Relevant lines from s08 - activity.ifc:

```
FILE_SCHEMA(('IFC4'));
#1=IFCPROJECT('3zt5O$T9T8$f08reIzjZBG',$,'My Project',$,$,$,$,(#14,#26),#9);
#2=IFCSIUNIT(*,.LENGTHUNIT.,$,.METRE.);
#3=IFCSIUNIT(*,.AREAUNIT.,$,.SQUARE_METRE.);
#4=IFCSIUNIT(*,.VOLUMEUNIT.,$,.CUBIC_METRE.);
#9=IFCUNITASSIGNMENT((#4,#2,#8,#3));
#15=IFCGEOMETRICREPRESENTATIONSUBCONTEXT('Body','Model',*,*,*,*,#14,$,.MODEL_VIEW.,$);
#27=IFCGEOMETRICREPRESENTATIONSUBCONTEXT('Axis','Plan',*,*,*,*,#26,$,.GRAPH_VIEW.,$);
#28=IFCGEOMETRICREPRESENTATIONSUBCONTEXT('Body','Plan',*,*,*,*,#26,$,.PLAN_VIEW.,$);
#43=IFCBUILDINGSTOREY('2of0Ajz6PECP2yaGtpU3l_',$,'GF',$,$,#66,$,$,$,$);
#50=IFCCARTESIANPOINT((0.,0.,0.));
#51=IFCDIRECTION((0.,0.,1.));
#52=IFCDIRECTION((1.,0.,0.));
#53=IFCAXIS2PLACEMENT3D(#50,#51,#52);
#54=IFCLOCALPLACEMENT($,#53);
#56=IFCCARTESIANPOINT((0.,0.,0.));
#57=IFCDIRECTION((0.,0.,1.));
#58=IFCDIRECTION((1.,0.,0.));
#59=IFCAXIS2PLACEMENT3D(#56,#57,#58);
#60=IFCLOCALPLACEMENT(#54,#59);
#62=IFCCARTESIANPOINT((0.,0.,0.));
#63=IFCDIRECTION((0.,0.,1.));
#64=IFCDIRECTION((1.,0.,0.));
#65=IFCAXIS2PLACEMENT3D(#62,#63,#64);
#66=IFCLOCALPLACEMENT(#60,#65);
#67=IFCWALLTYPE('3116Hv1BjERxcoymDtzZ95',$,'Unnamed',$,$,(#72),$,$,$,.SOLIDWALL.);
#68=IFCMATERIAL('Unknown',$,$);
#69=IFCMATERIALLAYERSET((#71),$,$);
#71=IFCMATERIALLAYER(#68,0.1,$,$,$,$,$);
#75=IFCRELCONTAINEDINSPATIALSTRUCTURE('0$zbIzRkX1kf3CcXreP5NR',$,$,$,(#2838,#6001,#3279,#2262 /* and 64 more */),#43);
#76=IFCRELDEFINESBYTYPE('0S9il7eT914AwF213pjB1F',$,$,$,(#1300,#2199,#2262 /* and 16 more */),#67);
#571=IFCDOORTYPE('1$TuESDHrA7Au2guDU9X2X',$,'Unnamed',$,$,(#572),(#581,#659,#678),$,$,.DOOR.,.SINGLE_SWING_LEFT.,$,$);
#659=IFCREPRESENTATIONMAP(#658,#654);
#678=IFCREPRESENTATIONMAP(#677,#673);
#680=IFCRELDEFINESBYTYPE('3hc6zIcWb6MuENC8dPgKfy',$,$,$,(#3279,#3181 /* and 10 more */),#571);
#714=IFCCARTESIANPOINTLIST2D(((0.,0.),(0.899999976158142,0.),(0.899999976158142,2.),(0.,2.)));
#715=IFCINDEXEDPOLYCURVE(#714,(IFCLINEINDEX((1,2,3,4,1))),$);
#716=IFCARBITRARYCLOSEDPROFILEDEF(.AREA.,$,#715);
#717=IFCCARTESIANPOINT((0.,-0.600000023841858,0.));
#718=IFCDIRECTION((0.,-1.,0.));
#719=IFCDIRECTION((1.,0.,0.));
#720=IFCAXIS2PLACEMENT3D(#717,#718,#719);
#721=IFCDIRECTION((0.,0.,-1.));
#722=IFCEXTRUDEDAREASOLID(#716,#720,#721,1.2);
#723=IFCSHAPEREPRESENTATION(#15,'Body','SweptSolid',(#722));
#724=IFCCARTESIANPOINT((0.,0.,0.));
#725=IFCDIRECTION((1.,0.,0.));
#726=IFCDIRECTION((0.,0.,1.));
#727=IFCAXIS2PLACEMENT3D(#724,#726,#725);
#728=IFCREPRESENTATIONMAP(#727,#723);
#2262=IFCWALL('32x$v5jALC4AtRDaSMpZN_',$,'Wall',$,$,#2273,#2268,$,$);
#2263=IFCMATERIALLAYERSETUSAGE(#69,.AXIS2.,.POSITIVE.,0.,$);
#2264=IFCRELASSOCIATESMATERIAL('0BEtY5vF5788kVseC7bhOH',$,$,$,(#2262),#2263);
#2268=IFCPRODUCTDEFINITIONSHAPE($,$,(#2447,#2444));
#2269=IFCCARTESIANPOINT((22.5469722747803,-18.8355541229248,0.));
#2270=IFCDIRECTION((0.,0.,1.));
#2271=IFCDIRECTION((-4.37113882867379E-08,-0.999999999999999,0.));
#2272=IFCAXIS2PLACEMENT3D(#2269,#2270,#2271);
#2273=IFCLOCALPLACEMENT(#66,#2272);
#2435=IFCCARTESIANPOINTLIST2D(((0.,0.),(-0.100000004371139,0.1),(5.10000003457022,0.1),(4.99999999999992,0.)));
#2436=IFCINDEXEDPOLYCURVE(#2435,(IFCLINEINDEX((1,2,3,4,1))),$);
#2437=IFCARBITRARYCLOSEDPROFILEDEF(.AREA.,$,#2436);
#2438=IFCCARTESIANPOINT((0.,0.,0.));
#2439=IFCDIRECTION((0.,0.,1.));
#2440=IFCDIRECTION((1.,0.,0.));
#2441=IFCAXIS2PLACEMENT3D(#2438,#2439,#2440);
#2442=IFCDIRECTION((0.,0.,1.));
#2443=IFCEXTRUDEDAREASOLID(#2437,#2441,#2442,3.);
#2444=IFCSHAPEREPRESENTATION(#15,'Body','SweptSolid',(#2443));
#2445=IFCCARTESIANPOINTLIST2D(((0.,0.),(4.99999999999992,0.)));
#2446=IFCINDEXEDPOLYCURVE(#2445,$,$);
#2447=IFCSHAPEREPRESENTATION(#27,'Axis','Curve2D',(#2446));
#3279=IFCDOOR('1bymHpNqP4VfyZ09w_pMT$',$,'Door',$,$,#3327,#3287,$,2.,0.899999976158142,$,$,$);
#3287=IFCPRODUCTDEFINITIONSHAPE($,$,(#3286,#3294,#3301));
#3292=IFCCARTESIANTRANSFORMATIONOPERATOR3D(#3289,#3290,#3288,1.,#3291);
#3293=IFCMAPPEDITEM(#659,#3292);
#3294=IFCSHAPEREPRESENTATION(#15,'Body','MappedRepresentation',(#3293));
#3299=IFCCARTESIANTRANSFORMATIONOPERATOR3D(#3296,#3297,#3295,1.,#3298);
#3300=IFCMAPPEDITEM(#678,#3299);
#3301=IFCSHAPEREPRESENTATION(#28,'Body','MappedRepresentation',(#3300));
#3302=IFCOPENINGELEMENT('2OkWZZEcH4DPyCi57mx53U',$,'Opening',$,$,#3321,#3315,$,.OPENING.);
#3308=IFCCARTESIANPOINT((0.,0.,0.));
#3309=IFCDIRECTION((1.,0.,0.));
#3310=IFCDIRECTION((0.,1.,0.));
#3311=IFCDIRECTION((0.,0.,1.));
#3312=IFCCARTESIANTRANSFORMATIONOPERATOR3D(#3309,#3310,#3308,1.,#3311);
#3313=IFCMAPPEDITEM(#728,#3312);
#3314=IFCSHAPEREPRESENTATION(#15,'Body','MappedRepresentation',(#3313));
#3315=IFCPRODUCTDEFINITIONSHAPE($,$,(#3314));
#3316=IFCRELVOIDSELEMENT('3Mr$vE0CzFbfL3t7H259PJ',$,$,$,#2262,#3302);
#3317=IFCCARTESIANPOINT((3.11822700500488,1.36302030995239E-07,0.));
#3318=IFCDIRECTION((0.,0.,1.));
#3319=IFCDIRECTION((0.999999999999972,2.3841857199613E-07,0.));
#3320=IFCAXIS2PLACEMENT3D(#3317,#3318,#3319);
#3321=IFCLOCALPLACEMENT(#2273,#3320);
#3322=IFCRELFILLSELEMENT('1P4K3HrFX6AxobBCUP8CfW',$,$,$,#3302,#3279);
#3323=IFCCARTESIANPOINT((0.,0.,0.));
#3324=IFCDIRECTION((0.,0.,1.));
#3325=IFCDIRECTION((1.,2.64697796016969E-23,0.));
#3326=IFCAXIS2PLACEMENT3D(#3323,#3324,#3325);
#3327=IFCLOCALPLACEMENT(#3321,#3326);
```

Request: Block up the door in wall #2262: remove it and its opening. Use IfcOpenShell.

```python
import ifcopenshell
import ifcopenshell.api.feature
import ifcopenshell.api.root
import ifcopenshell.geom
import ifcopenshell.util.shape

model = ifcopenshell.open("s08 - activity.ifc")
settings = ifcopenshell.geom.settings()


def volume(element):
    """Net volume in cubic metres, openings subtracted."""
    shape = ifcopenshell.geom.create_shape(settings, element)
    return ifcopenshell.util.shape.get_volume(shape.geometry)


door = model.by_id(3279)
opening = door.FillsVoids[0].RelatingOpeningElement
wall = opening.VoidsElements[0].RelatingBuildingElement
before = volume(wall)

ifcopenshell.api.root.remove_product(model, product=door)
ifcopenshell.api.feature.remove_feature(model, feature=opening)

after = volume(wall)

print(f"wall volume {before:.3f} -> {after:.3f} m3")

model.write("s08 - activity_edited.ifc")
```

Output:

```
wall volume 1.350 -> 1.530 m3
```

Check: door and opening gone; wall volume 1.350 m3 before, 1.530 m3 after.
